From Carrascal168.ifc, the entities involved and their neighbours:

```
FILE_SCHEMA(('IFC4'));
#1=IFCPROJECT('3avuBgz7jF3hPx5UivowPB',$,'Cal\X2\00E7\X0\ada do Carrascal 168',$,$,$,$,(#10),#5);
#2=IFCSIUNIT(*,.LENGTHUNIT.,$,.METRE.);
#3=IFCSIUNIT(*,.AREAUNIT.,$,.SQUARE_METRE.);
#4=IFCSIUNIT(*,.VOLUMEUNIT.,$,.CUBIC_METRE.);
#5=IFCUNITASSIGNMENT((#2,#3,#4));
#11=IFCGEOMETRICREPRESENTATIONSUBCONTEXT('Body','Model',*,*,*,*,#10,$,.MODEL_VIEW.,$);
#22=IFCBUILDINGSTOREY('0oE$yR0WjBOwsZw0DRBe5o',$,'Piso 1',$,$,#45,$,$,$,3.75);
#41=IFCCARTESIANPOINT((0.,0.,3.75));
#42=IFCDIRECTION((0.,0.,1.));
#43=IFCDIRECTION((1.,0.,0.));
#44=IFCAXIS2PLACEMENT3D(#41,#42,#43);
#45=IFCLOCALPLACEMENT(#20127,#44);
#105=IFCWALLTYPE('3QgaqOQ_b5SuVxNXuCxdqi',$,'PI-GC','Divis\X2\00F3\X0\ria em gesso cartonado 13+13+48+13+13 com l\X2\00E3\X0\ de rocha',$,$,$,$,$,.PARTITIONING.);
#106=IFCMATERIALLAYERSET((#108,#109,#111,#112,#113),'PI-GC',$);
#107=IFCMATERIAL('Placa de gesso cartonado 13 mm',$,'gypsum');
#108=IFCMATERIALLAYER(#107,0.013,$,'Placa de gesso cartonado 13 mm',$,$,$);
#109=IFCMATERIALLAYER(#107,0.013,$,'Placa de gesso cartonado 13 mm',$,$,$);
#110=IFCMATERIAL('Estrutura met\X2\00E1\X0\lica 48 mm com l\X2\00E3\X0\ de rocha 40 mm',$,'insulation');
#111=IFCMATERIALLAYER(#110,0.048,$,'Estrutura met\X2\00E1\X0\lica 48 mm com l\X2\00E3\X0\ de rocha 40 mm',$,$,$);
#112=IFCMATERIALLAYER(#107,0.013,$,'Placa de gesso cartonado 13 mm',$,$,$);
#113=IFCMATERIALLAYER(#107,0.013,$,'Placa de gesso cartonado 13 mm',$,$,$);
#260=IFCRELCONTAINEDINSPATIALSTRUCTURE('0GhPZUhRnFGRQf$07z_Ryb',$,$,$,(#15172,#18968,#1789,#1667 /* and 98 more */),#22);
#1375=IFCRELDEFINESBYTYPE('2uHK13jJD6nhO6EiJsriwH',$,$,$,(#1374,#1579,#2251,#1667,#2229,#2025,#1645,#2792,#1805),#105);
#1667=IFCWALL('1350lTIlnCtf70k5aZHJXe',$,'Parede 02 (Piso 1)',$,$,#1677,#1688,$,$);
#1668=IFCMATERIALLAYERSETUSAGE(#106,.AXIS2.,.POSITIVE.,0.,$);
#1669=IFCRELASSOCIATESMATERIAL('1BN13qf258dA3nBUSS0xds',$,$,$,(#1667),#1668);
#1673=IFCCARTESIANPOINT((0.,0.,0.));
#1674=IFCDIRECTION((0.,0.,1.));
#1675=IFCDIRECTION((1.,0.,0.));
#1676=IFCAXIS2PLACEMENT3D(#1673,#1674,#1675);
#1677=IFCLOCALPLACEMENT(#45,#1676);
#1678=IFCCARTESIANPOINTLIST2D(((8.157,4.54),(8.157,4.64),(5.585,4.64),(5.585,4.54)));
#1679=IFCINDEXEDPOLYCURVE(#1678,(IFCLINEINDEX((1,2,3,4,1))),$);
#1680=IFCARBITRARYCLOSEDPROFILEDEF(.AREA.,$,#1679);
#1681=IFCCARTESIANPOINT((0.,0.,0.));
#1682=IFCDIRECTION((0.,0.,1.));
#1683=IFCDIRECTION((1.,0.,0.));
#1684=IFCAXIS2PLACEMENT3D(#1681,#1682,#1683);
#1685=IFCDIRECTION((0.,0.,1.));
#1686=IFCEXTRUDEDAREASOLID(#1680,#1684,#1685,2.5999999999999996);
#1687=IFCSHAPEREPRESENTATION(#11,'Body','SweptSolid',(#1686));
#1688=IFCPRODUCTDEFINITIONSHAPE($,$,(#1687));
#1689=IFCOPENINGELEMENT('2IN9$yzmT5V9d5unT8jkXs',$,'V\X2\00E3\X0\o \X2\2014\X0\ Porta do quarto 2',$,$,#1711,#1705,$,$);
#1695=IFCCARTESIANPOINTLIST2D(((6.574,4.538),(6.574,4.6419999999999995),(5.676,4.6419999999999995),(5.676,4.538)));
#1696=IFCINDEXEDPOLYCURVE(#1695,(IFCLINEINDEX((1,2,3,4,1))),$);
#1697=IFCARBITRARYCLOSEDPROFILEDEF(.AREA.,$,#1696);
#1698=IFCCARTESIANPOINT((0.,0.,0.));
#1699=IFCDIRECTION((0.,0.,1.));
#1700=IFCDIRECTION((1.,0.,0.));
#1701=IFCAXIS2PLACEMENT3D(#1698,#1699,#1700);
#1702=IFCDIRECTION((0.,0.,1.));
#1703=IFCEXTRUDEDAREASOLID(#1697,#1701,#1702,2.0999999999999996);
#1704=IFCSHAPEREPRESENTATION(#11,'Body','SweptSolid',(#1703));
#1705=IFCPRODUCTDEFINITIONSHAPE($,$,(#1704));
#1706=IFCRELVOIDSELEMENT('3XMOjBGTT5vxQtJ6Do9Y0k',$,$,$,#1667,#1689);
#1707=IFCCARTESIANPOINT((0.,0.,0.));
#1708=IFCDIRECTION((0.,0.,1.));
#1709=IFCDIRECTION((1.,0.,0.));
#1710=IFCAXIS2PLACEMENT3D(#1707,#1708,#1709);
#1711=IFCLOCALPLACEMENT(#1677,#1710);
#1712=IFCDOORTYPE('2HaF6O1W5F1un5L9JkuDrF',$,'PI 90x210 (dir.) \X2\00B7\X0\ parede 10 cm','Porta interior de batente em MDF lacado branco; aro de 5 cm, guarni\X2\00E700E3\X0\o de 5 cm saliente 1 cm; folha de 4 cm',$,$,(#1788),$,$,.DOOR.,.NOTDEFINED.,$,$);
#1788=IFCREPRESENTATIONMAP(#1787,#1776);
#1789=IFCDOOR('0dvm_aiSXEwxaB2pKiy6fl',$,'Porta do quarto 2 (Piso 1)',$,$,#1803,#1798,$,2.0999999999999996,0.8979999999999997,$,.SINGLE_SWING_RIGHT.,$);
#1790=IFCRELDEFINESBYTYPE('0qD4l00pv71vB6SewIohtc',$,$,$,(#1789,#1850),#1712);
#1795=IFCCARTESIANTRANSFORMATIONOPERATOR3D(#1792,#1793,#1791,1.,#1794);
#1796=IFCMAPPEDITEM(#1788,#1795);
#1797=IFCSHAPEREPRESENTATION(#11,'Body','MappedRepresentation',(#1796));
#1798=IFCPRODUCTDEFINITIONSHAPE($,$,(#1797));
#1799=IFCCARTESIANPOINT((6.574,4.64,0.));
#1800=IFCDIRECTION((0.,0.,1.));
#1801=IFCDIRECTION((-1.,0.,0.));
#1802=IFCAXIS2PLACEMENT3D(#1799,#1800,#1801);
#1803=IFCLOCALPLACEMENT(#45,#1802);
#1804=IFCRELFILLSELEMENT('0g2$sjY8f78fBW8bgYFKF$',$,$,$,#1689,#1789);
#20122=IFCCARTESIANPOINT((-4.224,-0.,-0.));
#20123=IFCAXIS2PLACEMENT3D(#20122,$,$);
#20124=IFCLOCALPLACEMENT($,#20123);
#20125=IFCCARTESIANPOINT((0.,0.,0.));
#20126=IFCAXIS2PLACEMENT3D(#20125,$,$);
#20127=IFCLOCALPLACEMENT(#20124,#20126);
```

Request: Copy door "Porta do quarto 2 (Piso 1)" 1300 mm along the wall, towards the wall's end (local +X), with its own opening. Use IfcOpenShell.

```python
import ifcopenshell
import ifcopenshell.api.feature
import ifcopenshell.api.geometry
import ifcopenshell.api.root
import ifcopenshell.geom
import ifcopenshell.util.element
import ifcopenshell.util.placement
import ifcopenshell.util.shape

model = ifcopenshell.open("Carrascal168.ifc")
settings = ifcopenshell.geom.settings()


def volume(element):
    """Net volume in cubic metres, openings subtracted."""
    shape = ifcopenshell.geom.create_shape(settings, element)
    return ifcopenshell.util.shape.get_volume(shape.geometry)


door = model.by_id(1789)
opening = door.FillsVoids[0].RelatingOpeningElement
wall = opening.VoidsElements[0].RelatingBuildingElement
before = volume(wall)
shift = ifcopenshell.util.placement.get_local_placement(wall.ObjectPlacement)[:3, 0] * 1.3

# copy_class copies the void relationship, type, container and properties, but no geometry.
new_opening = ifcopenshell.api.root.copy_class(model, product=opening)
new_opening.Representation = ifcopenshell.util.element.copy_deep(
    model, opening.Representation, exclude=["IfcGeometricRepresentationContext", "IfcRepresentationMap"]
)
new_door = ifcopenshell.api.root.copy_class(model, product=door)
new_door.Representation = ifcopenshell.util.element.copy_deep(
    model, door.Representation, exclude=["IfcGeometricRepresentationContext", "IfcRepresentationMap"]
)
ifcopenshell.api.feature.add_filling(model, opening=new_opening, element=new_door)

for old, new in ((opening, new_opening), (door, new_door)):
    matrix = ifcopenshell.util.placement.get_local_placement(old.ObjectPlacement)
    matrix[:3, 3] += shift
    ifcopenshell.api.geometry.edit_object_placement(model, product=new, matrix=matrix, is_si=False)

after = volume(wall)

print(f"wall volume {before:.3f} -> {after:.3f} m3")

model.write("Carrascal168_v2.ifc")
```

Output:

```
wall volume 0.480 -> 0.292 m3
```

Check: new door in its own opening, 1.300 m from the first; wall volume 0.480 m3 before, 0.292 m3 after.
